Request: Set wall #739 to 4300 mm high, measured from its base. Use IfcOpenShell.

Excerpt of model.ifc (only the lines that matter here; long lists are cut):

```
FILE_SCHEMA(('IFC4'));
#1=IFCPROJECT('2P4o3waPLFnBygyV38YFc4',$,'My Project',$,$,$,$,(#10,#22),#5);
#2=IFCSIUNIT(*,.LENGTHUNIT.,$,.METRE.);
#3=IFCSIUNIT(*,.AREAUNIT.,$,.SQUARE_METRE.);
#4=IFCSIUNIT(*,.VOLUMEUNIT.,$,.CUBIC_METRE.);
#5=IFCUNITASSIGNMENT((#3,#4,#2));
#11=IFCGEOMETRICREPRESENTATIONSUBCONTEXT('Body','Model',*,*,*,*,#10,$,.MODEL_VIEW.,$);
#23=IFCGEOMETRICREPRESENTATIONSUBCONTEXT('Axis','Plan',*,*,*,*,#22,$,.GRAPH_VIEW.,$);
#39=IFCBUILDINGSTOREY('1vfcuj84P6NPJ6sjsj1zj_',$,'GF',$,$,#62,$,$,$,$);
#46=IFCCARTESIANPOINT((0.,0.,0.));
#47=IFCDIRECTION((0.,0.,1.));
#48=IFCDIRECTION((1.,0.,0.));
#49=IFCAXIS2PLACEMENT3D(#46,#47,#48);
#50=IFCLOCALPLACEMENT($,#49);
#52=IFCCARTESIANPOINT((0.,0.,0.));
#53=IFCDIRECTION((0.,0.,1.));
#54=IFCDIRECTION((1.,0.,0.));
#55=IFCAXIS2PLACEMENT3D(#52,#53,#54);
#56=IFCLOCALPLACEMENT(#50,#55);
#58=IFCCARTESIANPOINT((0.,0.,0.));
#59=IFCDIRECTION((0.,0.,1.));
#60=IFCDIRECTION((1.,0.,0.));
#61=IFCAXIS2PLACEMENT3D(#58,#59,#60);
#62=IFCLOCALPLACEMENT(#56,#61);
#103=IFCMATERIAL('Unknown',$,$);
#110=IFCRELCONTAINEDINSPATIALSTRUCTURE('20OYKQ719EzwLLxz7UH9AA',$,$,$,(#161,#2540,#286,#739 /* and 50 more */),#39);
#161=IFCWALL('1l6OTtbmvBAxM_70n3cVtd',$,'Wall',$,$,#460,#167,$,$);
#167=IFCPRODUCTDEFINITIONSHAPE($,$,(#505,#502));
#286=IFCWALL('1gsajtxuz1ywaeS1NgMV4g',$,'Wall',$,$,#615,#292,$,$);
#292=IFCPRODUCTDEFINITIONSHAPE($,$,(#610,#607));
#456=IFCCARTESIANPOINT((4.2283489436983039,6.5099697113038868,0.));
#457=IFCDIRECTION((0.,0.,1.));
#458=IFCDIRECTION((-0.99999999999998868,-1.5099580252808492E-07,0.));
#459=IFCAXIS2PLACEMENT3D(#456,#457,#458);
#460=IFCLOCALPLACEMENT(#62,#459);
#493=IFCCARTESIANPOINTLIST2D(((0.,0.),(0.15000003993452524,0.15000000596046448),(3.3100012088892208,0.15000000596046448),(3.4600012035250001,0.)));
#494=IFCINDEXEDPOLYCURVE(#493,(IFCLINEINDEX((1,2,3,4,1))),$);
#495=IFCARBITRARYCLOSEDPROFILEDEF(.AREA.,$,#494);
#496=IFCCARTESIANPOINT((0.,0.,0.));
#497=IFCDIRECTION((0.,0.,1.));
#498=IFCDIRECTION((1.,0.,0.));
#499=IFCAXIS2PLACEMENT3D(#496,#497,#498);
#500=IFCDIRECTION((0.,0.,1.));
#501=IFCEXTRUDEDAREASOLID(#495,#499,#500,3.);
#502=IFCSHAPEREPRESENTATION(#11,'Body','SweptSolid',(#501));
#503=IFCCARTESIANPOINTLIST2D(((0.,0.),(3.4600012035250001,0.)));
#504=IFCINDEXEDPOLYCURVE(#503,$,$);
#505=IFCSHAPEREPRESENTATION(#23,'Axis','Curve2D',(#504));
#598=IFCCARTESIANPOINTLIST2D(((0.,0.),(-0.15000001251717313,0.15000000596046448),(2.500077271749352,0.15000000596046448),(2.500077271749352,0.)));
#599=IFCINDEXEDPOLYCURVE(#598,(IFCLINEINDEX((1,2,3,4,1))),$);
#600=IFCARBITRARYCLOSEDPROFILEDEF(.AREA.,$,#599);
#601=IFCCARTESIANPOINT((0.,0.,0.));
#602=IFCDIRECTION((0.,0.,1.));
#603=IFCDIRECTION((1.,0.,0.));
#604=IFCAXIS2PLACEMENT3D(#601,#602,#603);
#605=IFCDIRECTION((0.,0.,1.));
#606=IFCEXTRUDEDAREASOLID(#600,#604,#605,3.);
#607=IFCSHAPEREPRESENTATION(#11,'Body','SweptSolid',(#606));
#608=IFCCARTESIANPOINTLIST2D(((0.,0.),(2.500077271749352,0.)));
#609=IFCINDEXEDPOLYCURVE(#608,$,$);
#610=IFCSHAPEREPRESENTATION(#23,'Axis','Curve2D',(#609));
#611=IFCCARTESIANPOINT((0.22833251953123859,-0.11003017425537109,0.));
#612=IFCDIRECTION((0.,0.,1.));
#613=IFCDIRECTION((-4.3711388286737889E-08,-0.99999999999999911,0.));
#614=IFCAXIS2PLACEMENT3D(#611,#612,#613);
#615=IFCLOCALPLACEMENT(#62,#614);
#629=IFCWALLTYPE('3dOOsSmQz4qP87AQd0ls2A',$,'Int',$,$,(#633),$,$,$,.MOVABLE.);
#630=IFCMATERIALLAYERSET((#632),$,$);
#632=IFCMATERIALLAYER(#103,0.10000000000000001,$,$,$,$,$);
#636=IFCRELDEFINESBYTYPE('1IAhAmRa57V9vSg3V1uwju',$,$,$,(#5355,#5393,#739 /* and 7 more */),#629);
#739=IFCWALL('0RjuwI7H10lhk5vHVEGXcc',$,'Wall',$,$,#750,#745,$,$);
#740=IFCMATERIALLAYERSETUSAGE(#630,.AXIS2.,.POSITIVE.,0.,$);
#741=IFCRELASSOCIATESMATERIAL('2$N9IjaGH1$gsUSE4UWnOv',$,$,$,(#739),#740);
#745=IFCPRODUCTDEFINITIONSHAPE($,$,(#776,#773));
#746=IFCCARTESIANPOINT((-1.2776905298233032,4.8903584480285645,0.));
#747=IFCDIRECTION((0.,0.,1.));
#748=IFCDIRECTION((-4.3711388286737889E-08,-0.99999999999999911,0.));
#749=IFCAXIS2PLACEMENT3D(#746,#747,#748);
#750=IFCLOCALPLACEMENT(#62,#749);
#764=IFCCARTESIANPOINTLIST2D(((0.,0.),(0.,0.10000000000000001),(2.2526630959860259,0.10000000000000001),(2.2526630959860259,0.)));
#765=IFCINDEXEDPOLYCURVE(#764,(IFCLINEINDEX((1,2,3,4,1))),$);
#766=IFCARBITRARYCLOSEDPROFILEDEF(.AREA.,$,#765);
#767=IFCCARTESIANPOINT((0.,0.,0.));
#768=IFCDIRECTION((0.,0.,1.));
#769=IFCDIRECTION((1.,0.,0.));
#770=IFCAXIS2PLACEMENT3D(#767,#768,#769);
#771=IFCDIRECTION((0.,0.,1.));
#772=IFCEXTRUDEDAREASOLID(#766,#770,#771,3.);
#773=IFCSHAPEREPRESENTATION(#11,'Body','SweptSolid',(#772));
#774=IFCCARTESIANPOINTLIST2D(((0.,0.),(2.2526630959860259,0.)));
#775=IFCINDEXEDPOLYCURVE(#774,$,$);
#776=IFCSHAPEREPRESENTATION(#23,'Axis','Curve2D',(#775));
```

```python
import ifcopenshell
import ifcopenshell.geom
import ifcopenshell.util.representation
import ifcopenshell.util.shape
import ifcopenshell.util.unit

model = ifcopenshell.open("model.ifc")
unit_scale = ifcopenshell.util.unit.calculate_unit_scale(model)
settings = ifcopenshell.geom.settings()


def volume(element):
    """Net volume in cubic metres, openings subtracted."""
    shape = ifcopenshell.geom.create_shape(settings, element)
    return ifcopenshell.util.shape.get_volume(shape.geometry)


wall = model.by_id(739)
before = volume(wall)

body = ifcopenshell.util.representation.get_representation(wall, "Model", "Body")
solid = body.Items[0]
old_height = solid.Depth
solid.Depth = 4.3 / unit_scale
after = volume(wall)

print(f"height {old_height:g} -> {solid.Depth:g}, volume {before:.3f} -> {after:.3f} m3")

model.write("model_updated.ifc")
```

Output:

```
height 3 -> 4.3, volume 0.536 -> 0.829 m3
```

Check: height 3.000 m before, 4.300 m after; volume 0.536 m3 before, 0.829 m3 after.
